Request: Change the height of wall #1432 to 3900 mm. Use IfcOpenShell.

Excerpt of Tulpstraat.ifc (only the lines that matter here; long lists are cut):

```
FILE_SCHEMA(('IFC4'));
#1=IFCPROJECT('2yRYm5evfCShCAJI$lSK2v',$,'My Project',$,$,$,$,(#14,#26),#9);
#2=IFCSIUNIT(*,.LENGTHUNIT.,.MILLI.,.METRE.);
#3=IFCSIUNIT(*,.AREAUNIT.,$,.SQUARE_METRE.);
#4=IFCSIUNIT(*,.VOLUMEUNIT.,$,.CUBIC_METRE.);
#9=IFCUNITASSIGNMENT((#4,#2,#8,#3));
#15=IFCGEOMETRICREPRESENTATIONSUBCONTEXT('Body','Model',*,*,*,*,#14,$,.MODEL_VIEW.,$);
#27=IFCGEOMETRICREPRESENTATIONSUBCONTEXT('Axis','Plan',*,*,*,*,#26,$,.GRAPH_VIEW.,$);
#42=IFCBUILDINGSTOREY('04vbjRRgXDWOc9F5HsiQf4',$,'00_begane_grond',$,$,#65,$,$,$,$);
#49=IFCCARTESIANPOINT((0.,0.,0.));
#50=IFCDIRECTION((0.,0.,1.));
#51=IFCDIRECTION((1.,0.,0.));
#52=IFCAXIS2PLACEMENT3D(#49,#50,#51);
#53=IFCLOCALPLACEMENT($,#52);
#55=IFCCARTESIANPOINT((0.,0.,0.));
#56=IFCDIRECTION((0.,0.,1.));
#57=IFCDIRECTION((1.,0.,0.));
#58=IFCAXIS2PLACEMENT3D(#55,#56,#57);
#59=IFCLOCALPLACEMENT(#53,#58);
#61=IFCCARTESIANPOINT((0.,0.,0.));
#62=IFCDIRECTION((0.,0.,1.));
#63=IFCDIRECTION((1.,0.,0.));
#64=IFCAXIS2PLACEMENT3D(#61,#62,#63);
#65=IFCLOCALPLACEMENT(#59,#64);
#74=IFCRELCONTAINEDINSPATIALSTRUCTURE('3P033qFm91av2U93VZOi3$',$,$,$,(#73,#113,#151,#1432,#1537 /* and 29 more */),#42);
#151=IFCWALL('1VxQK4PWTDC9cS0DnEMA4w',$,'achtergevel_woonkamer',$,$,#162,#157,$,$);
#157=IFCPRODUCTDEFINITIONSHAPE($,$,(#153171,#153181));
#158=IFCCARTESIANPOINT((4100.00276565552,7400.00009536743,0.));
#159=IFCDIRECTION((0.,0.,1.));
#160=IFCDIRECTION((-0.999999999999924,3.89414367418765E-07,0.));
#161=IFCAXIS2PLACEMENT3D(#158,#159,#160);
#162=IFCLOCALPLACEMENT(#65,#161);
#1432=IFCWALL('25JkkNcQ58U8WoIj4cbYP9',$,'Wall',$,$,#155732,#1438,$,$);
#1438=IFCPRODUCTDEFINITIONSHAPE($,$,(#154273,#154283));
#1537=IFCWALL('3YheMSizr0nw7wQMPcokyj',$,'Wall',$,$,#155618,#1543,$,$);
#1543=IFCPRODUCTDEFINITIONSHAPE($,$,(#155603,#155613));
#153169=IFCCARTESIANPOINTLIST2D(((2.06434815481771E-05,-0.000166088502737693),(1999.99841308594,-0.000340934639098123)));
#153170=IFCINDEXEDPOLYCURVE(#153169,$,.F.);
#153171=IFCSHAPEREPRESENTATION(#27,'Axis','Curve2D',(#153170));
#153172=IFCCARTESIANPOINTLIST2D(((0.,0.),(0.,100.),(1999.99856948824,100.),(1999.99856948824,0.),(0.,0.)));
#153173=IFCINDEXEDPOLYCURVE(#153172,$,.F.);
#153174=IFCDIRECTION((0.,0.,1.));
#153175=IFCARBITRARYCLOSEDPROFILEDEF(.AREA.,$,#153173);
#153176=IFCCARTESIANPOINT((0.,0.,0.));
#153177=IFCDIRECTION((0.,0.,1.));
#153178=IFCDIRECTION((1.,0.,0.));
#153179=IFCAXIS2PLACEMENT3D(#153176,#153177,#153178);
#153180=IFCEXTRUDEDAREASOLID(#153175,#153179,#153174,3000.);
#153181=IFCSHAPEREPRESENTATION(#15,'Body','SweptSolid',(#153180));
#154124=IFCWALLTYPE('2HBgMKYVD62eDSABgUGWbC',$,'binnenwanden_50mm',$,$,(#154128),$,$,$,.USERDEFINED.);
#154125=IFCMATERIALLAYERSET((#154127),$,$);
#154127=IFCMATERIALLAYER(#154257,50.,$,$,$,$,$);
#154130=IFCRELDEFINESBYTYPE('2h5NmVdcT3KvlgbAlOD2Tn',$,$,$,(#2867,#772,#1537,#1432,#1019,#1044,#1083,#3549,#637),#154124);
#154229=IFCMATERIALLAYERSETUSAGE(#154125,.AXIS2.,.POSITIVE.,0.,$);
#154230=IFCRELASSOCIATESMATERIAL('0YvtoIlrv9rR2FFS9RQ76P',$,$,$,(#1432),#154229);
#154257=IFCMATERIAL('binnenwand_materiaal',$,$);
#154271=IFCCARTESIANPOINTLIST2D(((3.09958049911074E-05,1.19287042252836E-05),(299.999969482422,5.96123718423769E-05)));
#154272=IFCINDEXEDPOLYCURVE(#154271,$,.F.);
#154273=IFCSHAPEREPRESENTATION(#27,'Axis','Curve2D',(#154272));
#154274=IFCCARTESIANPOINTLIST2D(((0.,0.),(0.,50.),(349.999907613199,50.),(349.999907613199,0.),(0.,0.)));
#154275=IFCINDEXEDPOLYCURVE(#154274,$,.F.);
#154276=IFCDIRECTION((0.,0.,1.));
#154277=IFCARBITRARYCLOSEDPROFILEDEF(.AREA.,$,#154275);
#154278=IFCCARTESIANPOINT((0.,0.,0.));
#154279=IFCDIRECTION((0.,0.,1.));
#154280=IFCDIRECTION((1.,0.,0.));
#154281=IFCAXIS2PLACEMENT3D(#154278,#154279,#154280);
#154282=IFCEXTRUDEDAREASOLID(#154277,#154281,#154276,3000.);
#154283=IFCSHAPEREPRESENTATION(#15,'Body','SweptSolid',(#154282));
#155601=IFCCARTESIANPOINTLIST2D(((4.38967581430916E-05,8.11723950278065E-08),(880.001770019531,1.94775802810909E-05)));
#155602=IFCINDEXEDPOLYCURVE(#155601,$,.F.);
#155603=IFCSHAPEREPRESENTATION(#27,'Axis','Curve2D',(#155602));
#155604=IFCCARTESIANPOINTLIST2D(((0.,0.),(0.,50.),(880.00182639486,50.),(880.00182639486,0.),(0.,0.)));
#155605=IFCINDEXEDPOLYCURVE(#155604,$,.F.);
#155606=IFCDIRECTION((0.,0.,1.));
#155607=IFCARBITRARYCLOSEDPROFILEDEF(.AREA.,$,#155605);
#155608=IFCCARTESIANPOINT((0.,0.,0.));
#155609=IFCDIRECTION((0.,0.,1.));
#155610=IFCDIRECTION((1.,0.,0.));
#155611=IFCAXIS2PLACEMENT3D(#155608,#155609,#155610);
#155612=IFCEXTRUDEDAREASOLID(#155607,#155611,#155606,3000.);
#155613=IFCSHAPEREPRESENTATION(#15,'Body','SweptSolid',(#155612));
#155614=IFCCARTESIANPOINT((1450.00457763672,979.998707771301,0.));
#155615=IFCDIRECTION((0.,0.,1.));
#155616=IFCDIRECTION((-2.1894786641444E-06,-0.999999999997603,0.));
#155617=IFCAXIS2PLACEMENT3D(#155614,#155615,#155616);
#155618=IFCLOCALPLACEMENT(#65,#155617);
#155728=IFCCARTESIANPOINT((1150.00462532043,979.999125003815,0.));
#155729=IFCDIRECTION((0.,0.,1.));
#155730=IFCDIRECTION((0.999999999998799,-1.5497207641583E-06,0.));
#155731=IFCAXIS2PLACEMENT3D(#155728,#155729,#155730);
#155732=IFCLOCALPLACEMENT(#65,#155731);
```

```python
import ifcopenshell
import ifcopenshell.geom
import ifcopenshell.util.representation
import ifcopenshell.util.shape
import ifcopenshell.util.unit

model = ifcopenshell.open("Tulpstraat.ifc")
unit_scale = ifcopenshell.util.unit.calculate_unit_scale(model)
settings = ifcopenshell.geom.settings()


def volume(element):
    """Net volume in cubic metres, openings subtracted."""
    shape = ifcopenshell.geom.create_shape(settings, element)
    return ifcopenshell.util.shape.get_volume(shape.geometry)


wall = model.by_id(1432)
before = volume(wall)

body = ifcopenshell.util.representation.get_representation(wall, "Model", "Body")
solid = body.Items[0]
old_height = solid.Depth
solid.Depth = 3.9 / unit_scale
after = volume(wall)

print(f"height {old_height:g} -> {solid.Depth:g}, volume {before:.3f} -> {after:.3f} m3")

model.write("Tulpstraat_updated.ifc")
```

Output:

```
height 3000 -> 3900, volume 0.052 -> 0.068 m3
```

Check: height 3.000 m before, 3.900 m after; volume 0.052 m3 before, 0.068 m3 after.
